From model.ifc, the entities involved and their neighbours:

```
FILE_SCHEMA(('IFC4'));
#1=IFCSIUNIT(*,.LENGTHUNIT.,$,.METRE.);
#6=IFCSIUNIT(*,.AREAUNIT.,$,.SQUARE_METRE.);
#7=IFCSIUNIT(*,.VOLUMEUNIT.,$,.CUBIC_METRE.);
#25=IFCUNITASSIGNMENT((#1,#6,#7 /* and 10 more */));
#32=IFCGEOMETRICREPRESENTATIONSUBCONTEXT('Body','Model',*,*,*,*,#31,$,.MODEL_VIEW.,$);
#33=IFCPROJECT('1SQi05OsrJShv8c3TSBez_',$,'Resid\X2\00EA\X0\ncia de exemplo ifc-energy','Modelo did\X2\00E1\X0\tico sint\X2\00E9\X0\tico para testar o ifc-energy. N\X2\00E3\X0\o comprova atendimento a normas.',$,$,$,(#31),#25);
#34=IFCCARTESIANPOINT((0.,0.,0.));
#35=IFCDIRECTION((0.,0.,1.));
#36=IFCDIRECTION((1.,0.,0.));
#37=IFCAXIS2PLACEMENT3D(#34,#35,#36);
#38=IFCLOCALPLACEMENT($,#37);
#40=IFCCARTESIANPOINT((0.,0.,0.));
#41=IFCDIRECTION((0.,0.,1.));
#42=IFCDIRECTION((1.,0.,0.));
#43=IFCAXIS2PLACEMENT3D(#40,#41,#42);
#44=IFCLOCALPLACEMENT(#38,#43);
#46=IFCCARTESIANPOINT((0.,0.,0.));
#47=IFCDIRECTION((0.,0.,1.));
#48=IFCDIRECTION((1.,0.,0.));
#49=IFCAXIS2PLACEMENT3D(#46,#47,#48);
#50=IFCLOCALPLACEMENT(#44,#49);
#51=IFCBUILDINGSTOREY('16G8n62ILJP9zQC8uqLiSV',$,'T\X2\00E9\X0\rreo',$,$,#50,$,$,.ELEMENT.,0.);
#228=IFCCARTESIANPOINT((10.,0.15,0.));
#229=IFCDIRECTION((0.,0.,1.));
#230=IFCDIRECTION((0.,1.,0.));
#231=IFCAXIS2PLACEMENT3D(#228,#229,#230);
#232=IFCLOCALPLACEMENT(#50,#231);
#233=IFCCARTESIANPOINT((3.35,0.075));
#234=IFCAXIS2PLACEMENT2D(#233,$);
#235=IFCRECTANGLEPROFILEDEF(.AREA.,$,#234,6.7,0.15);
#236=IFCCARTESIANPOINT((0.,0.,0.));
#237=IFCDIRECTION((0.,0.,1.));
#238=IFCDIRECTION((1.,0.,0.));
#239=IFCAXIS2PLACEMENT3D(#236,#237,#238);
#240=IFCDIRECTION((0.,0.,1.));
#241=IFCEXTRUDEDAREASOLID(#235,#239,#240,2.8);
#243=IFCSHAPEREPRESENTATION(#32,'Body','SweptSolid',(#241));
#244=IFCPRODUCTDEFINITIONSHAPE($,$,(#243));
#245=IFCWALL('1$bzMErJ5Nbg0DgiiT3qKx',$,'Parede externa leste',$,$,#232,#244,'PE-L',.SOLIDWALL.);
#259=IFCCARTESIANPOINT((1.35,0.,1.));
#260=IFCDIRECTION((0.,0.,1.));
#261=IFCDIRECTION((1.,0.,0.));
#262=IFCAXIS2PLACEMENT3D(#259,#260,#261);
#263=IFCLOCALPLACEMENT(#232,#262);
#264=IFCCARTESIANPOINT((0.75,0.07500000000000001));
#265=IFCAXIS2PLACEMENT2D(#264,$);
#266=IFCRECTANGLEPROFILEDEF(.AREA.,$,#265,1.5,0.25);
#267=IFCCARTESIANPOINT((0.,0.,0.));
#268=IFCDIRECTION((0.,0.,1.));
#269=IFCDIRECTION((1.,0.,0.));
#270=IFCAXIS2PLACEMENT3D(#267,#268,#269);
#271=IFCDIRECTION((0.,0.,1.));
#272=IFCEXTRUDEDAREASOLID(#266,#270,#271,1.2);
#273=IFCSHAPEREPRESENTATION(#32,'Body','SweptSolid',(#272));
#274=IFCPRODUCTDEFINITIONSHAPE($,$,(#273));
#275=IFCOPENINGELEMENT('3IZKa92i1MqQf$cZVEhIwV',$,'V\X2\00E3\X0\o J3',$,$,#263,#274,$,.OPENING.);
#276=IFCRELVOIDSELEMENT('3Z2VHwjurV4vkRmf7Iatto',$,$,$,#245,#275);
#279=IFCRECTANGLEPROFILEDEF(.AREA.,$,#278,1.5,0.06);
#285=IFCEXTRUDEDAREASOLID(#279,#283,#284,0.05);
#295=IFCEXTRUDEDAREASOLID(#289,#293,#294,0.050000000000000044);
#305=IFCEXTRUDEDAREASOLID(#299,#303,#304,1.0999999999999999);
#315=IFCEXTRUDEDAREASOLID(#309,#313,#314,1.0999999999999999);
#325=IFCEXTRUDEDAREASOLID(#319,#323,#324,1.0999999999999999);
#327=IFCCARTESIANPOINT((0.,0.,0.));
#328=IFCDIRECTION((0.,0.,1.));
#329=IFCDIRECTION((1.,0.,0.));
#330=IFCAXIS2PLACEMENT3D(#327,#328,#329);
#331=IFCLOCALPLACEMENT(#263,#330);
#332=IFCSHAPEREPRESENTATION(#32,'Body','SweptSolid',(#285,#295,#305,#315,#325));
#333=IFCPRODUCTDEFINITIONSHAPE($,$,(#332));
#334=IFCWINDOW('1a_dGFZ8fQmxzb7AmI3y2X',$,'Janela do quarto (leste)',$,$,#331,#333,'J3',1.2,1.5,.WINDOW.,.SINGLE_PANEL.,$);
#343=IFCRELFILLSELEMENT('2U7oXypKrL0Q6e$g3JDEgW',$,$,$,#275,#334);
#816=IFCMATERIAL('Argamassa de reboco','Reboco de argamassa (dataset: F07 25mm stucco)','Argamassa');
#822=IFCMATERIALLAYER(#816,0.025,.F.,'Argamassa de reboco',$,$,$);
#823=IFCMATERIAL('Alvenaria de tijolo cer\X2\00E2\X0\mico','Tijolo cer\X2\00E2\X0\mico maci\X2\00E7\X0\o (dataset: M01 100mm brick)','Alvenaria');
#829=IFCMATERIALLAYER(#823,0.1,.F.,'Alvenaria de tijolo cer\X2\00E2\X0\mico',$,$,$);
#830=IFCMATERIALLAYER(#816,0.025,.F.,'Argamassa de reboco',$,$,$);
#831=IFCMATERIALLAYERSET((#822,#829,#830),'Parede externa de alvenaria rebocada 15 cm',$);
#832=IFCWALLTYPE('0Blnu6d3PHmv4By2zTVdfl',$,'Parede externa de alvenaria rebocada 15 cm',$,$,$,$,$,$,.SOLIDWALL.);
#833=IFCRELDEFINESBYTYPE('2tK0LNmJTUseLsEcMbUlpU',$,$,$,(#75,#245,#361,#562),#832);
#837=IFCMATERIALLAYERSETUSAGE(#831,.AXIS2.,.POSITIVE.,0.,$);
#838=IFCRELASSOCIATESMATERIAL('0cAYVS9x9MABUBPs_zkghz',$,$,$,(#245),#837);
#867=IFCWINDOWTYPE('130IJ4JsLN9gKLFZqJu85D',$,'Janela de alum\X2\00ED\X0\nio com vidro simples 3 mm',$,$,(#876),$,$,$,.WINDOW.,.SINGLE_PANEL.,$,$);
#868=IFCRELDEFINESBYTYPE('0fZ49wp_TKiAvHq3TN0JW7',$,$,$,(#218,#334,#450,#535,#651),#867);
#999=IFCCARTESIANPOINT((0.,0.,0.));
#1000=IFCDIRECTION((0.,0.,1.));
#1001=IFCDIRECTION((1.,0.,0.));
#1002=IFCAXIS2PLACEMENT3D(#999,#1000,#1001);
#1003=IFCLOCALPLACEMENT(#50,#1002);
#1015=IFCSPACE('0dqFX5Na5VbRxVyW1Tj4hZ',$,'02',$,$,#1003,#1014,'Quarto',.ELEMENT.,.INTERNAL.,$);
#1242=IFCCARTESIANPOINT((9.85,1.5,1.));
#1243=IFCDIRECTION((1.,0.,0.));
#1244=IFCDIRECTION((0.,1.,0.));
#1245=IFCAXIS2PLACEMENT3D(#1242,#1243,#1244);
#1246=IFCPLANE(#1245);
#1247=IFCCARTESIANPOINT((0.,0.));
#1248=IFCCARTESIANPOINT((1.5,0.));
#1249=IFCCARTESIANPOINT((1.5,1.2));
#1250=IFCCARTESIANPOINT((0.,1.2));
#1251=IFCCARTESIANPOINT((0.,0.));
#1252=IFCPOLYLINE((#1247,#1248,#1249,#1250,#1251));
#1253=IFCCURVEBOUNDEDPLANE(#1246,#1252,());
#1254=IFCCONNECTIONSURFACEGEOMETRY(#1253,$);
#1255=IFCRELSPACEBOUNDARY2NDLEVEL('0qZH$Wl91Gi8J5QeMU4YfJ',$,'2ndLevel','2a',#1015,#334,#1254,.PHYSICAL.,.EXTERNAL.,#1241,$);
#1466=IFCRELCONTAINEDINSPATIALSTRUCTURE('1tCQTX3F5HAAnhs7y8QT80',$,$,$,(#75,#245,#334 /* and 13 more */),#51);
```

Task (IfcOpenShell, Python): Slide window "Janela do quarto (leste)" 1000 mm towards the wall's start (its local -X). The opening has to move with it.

```python
import numpy as np
import ifcopenshell
import ifcopenshell.api.geometry
import ifcopenshell.util.placement
import ifcopenshell.util.unit

model = ifcopenshell.open("model.ifc")
unit_scale = ifcopenshell.util.unit.calculate_unit_scale(model)

window = model.by_guid("1a_dGFZ8fQmxzb7AmI3y2X")
opening = window.FillsVoids[0].RelatingOpeningElement
wall = opening.VoidsElements[0].RelatingBuildingElement

wall_matrix = ifcopenshell.util.placement.get_local_placement(wall.ObjectPlacement)
shift = wall_matrix[:3, 0] * -1 / unit_scale
before = ifcopenshell.util.placement.get_local_placement(window.ObjectPlacement)[:3, 3].copy()

# The window is placed relative to its opening, so it follows when the opening moves.
matrix = ifcopenshell.util.placement.get_local_placement(opening.ObjectPlacement)
matrix[:3, 3] += shift
ifcopenshell.api.geometry.edit_object_placement(
    model, product=opening, matrix=matrix, is_si=False, should_transform_children=True
)

# Space boundary surfaces are stored in each space's coordinates; move them too.
for rel in window.ProvidesBoundaries:
    if not rel.ConnectionGeometry:
        continue
    surface = rel.ConnectionGeometry.SurfaceOnRelatingElement.BasisSurface
    space_matrix = ifcopenshell.util.placement.get_local_placement(rel.RelatingSpace.ObjectPlacement)
    point = np.array(surface.Position.Location.Coordinates) + space_matrix[:3, :3].T @ shift
    surface.Position = model.createIfcAxis2Placement3D(
        model.createIfcCartesianPoint(point.tolist()), surface.Position.Axis, surface.Position.RefDirection
    )

after = ifcopenshell.util.placement.get_local_placement(window.ObjectPlacement)[:3, 3]
print("window moved by", (after - before).round(3) + 0.0)

model.write("model_v2.ifc")
```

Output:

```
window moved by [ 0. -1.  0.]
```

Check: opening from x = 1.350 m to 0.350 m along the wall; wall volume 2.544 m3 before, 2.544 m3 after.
